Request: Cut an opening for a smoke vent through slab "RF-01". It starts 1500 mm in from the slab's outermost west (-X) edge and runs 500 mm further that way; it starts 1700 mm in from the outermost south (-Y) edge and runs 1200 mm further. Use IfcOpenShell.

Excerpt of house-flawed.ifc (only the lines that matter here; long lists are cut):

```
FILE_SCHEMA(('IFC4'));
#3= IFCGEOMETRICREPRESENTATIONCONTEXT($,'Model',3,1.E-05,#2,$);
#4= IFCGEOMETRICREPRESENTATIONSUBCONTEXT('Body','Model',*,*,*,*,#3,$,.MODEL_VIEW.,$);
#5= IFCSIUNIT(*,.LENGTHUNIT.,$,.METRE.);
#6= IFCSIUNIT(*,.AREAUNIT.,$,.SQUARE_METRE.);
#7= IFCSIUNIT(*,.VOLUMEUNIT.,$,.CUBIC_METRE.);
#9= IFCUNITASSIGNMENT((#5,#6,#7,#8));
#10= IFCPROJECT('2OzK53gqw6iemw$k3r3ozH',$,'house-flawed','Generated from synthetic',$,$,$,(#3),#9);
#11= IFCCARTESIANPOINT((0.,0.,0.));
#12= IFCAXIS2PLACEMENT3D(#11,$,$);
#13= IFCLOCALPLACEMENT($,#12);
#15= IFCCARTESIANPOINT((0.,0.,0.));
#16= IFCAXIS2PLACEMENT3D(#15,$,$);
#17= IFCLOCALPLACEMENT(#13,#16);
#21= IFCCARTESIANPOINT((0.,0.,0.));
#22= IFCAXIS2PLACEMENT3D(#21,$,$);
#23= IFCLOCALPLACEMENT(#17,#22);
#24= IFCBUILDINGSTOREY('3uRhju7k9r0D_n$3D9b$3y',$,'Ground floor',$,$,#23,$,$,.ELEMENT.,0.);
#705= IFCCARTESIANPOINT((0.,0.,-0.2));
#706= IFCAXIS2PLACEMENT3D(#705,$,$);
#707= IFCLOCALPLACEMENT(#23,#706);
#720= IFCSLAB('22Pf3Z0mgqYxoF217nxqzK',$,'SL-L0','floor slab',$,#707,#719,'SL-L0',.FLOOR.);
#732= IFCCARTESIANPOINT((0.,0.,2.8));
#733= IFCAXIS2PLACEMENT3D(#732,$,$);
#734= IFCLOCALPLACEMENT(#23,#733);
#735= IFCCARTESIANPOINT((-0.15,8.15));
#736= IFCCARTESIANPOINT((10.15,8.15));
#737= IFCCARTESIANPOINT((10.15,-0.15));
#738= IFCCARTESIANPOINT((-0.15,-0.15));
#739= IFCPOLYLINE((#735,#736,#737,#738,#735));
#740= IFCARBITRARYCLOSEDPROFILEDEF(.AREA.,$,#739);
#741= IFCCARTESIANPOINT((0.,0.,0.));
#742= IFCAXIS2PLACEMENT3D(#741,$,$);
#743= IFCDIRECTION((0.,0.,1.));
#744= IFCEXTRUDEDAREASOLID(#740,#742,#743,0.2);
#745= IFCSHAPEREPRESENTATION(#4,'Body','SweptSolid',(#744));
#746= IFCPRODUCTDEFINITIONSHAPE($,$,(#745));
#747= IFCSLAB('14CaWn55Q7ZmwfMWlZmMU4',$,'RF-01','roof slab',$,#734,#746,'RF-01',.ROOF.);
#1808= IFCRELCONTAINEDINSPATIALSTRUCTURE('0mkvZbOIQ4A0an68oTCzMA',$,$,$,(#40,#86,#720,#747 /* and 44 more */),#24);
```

```python
import numpy as np
import ifcopenshell
import ifcopenshell.api.feature
import ifcopenshell.api.geometry
import ifcopenshell.api.root
import ifcopenshell.geom
import ifcopenshell.util.placement
import ifcopenshell.util.representation
import ifcopenshell.util.shape
import ifcopenshell.util.unit

model = ifcopenshell.open("house-flawed.ifc")
unit_scale = ifcopenshell.util.unit.calculate_unit_scale(model)
settings = ifcopenshell.geom.settings()


def volume(element):
    """Net volume in cubic metres, openings subtracted."""
    shape = ifcopenshell.geom.create_shape(settings, element)
    return ifcopenshell.util.shape.get_volume(shape.geometry)


slab = model.by_guid("14CaWn55Q7ZmwfMWlZmMU4")
before = volume(slab)

# Extent in the slab's own axes, in metres. The edges named are its -X and -Y sides.
slab_shape = ifcopenshell.geom.create_shape(settings, slab)
vertices = ifcopenshell.util.shape.get_vertices(slab_shape.geometry)
x_min, y_min, bottom = vertices.min(axis=0)
top = vertices[:, 2].max()

opening = ifcopenshell.api.root.create_entity(model, ifc_class="IfcOpeningElement", name="Smoke vent opening", predefined_type="OPENING")
context = ifcopenshell.util.representation.get_context(model, "Model", "Body", "MODEL_VIEW")
width, depth = 0.5, 1.2
outline = [(0.0, 0.0), (width, 0.0), (width, depth), (0.0, depth), (0.0, 0.0)]
# Overshoot both faces by 50 mm so the cut is clean.
shape = ifcopenshell.api.geometry.add_slab_representation(
    model, context=context, depth=top - bottom + 0.1, polyline=outline
)
ifcopenshell.api.geometry.assign_representation(model, product=opening, representation=shape)

matrix = ifcopenshell.util.placement.get_local_placement(slab.ObjectPlacement)
matrix[:, 3] = matrix @ np.append(np.array([x_min + 1.5, y_min + 1.7, bottom - 0.05]) / unit_scale, 1.0)
ifcopenshell.api.geometry.edit_object_placement(model, product=opening, matrix=matrix, is_si=False)
ifcopenshell.api.feature.add_feature(model, feature=opening, element=slab)

after = volume(slab)

print(f"slab volume {before:.3f} -> {after:.3f} m3")

model.write("house-flawed_v2.ifc")
```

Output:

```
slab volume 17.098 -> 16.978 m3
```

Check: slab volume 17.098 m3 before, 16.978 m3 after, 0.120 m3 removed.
